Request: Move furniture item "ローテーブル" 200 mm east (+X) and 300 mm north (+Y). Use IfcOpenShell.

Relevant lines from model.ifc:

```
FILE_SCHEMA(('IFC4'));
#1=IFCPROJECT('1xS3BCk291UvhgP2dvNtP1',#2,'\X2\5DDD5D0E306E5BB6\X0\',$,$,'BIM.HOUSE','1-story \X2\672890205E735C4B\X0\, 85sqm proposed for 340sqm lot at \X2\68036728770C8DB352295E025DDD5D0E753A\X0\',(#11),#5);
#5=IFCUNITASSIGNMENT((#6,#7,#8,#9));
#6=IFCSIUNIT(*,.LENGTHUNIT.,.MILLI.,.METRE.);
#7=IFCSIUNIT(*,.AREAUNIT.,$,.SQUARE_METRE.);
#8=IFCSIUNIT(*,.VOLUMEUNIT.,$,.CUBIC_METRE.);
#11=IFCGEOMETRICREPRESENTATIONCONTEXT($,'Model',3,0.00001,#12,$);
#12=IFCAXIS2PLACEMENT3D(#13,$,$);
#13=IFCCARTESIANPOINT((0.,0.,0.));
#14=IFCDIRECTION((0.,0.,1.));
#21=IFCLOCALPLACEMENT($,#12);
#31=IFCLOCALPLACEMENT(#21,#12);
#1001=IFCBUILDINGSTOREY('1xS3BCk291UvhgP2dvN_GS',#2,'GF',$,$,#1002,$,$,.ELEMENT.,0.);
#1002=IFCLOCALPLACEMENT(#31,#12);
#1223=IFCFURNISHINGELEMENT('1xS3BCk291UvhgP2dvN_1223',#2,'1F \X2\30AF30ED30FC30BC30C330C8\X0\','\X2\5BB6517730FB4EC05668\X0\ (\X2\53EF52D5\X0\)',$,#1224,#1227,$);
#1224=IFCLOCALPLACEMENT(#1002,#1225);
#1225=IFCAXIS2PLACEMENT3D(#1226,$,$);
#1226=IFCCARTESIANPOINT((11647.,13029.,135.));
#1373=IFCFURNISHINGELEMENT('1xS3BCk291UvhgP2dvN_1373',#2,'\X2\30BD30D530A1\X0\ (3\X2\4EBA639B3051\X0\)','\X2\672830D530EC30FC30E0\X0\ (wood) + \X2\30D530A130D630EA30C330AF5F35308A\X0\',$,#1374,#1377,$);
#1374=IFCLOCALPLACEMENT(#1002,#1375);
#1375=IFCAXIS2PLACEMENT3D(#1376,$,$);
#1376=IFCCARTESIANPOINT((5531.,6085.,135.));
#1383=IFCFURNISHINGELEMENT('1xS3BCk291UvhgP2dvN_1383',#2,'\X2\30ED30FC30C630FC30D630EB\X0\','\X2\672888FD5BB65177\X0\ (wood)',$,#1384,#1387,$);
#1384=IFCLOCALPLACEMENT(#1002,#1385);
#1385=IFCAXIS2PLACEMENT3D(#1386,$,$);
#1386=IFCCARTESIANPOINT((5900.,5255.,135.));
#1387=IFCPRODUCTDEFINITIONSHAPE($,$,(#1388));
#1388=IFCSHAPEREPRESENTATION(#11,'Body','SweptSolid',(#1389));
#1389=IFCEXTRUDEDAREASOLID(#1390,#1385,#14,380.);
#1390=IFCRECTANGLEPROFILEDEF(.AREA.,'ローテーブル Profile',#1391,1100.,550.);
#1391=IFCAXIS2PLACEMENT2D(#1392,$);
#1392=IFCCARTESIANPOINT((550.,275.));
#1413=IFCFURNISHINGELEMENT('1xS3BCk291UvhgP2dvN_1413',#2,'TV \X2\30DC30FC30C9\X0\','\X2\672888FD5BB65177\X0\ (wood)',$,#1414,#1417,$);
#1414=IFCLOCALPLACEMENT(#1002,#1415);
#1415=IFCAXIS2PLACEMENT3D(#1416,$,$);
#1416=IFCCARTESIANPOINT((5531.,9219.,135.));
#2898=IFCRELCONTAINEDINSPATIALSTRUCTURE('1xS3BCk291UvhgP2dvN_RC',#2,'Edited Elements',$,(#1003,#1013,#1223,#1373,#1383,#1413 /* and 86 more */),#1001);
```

```python
import ifcopenshell
import ifcopenshell.api.geometry
import ifcopenshell.util.placement
import ifcopenshell.util.unit

model = ifcopenshell.open("model.ifc")
unit_scale = ifcopenshell.util.unit.calculate_unit_scale(model)

item = model.by_guid("1xS3BCk291UvhgP2dvN_1383")
matrix = ifcopenshell.util.placement.get_local_placement(item.ObjectPlacement)
matrix[0, 3] += 0.2 / unit_scale
matrix[1, 3] += 0.3 / unit_scale
ifcopenshell.api.geometry.edit_object_placement(model, product=item, matrix=matrix, is_si=False)

print(ifcopenshell.util.placement.get_local_placement(item.ObjectPlacement).round(3) + 0.0)

model.write("model-out.ifc")
```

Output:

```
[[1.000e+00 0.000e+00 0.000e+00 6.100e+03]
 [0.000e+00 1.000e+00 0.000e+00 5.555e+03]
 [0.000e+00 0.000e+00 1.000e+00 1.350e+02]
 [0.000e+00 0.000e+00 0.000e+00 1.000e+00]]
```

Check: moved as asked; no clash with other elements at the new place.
